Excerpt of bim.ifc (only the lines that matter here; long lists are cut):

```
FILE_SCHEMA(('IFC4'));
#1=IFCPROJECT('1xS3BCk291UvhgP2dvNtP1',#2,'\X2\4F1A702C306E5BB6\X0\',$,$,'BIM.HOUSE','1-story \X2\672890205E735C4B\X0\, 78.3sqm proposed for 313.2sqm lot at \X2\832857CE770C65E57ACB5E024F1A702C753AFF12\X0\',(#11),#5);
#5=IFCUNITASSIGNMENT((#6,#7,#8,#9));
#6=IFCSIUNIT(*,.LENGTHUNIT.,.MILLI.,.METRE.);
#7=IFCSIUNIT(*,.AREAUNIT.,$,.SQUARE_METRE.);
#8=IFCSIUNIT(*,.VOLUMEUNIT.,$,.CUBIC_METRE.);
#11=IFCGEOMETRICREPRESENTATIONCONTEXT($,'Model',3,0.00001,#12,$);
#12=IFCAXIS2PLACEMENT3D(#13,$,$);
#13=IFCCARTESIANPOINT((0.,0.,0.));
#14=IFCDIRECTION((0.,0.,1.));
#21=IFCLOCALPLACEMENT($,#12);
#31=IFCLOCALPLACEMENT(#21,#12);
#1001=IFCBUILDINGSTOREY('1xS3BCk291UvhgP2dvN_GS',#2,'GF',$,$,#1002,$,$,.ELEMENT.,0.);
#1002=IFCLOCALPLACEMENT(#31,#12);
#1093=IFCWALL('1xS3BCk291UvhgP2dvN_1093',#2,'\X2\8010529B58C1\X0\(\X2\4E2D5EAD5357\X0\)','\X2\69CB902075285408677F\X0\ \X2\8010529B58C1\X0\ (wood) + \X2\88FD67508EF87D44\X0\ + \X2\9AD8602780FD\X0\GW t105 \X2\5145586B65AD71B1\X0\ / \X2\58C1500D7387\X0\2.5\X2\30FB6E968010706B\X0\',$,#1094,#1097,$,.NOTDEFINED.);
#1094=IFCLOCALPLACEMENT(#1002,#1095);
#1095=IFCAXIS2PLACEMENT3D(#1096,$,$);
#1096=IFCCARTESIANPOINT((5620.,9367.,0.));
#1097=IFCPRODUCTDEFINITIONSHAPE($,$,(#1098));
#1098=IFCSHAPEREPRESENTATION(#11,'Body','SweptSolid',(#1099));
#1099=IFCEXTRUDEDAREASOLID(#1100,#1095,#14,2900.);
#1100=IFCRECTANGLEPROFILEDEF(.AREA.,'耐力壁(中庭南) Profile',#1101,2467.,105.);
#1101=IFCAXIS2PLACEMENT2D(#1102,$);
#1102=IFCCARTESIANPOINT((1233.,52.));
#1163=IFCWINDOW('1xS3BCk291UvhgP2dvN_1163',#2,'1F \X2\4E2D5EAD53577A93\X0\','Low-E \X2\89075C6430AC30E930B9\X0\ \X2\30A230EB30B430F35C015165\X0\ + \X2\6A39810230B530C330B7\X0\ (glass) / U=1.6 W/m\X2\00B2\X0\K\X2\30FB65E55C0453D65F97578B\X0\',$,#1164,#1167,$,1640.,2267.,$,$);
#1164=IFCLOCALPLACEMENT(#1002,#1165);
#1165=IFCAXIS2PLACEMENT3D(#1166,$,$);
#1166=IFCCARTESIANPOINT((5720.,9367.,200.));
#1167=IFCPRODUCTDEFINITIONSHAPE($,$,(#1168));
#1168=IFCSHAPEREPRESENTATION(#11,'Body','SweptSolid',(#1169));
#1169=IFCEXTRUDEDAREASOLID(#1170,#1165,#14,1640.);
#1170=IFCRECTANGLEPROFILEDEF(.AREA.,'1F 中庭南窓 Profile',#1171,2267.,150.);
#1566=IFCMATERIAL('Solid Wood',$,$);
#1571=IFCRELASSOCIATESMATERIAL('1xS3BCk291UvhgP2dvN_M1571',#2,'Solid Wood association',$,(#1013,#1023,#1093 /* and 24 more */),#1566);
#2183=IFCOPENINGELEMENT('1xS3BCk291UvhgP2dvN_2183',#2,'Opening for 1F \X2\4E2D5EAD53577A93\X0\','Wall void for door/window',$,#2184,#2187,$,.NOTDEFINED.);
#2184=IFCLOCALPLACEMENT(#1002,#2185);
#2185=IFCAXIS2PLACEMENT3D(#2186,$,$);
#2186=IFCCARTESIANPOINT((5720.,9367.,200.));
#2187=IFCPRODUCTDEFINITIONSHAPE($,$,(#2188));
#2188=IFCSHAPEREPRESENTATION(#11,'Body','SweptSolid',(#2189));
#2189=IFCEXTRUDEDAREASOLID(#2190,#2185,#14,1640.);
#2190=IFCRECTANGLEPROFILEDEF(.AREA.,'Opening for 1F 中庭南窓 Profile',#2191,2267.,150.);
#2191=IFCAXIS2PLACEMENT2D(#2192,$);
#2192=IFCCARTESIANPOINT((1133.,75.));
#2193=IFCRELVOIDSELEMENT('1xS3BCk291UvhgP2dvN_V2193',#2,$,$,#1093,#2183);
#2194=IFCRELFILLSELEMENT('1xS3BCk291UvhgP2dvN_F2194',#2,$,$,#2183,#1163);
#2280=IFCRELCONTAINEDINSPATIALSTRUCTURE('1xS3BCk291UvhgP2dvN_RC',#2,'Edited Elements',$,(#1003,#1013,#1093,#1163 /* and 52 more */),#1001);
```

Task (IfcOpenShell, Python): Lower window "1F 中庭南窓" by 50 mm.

```python
import numpy as np
import ifcopenshell
import ifcopenshell.api.geometry
import ifcopenshell.util.placement
import ifcopenshell.util.unit

model = ifcopenshell.open("bim.ifc")
unit_scale = ifcopenshell.util.unit.calculate_unit_scale(model)

window = model.by_guid("1xS3BCk291UvhgP2dvN_1163")
opening = window.FillsVoids[0].RelatingOpeningElement
dz = -0.05 / unit_scale

shift = np.array([0.0, 0.0, dz])
# The window is not placed relative to its opening, so move both.
for product in (opening, window):
    matrix = ifcopenshell.util.placement.get_local_placement(product.ObjectPlacement)
    matrix[:3, 3] += shift
    ifcopenshell.api.geometry.edit_object_placement(model, product=product, matrix=matrix, is_si=False)

print(f"moved by {dz * unit_scale:+.3f} m")

model.write("bim_edited.ifc")
```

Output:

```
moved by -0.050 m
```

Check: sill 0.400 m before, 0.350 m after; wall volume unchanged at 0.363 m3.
